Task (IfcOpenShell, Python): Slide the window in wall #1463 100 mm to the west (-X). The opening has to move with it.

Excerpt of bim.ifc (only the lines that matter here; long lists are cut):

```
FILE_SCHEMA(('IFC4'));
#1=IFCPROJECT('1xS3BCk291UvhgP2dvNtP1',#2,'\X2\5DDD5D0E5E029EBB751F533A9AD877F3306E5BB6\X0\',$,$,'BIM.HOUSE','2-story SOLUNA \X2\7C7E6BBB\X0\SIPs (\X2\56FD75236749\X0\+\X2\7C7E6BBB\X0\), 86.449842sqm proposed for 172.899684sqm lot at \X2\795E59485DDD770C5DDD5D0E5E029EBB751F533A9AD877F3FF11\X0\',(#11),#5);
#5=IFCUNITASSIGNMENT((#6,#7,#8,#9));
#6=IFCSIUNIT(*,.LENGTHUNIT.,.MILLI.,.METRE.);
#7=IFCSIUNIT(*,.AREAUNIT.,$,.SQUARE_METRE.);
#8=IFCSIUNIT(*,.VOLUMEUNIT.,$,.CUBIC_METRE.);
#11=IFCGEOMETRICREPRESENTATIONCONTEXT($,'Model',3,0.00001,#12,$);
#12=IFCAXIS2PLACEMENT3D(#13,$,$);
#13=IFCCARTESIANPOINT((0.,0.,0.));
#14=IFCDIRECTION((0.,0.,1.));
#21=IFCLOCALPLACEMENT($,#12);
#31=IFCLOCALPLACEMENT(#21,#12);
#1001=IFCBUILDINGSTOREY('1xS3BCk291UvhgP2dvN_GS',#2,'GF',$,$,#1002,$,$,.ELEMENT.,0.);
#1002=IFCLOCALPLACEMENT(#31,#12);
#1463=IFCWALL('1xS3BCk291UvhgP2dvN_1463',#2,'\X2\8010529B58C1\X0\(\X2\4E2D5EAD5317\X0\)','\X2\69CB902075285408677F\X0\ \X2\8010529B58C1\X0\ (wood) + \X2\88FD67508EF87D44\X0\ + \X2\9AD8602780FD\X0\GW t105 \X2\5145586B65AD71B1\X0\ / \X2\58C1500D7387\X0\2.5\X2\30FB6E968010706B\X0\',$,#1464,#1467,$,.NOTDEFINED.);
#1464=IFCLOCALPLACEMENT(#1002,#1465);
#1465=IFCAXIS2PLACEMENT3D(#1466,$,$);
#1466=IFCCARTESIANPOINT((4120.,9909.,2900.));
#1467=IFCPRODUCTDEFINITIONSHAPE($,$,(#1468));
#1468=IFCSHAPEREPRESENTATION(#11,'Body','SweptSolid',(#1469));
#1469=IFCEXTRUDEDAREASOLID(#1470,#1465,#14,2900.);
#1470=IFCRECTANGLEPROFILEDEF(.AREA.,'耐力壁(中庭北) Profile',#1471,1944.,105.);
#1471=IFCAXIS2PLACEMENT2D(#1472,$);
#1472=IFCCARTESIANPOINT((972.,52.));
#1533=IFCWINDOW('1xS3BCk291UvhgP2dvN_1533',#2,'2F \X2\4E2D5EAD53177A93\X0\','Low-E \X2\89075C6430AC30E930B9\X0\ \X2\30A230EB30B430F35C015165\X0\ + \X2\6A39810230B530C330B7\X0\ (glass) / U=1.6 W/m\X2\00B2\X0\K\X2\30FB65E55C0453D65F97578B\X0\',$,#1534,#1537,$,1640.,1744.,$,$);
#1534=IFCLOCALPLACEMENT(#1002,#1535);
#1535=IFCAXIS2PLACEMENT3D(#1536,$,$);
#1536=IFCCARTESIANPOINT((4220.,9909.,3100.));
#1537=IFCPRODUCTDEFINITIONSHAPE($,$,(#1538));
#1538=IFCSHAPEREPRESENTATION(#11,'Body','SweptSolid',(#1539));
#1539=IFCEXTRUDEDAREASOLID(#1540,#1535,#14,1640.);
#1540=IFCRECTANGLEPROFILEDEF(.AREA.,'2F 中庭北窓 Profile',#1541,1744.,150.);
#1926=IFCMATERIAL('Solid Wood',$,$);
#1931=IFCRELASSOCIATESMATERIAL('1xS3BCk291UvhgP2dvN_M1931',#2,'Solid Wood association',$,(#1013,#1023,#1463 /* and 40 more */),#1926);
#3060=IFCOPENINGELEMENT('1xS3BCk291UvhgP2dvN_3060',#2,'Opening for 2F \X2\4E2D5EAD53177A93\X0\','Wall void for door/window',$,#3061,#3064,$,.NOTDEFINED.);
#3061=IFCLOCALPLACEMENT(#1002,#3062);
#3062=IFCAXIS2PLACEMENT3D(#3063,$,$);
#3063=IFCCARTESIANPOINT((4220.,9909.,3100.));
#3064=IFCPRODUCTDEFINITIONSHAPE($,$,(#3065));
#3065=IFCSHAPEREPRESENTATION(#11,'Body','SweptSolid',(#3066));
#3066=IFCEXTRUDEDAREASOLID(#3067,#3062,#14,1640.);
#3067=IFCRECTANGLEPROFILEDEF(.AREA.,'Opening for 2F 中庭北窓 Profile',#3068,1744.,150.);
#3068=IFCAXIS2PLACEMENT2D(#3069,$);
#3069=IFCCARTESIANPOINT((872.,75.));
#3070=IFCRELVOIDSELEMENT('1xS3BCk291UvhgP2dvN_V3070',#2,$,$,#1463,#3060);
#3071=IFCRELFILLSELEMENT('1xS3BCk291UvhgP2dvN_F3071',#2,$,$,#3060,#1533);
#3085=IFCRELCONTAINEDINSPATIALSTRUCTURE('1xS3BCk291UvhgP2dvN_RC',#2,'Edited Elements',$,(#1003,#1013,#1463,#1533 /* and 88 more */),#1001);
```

```python
import ifcopenshell
import ifcopenshell.api.geometry
import ifcopenshell.util.placement
import ifcopenshell.util.unit

model = ifcopenshell.open("bim.ifc")
unit_scale = ifcopenshell.util.unit.calculate_unit_scale(model)

window = model.by_guid("1xS3BCk291UvhgP2dvN_1533")
opening = window.FillsVoids[0].RelatingOpeningElement
wall = opening.VoidsElements[0].RelatingBuildingElement

wall_matrix = ifcopenshell.util.placement.get_local_placement(wall.ObjectPlacement)
shift = wall_matrix[:3, 0] * -0.1 / unit_scale
before = ifcopenshell.util.placement.get_local_placement(window.ObjectPlacement)[:3, 3].copy()

# The window is not placed relative to its opening, so move both.
for product in (opening, window):
    matrix = ifcopenshell.util.placement.get_local_placement(product.ObjectPlacement)
    matrix[:3, 3] += shift
    ifcopenshell.api.geometry.edit_object_placement(model, product=product, matrix=matrix, is_si=False)

after = ifcopenshell.util.placement.get_local_placement(window.ObjectPlacement)[:3, 3]
print("window moved by", (after - before).round(3) + 0.0)

model.write("bim_edited.ifc")
```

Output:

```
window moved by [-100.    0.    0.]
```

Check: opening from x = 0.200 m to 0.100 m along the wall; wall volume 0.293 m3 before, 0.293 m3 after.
